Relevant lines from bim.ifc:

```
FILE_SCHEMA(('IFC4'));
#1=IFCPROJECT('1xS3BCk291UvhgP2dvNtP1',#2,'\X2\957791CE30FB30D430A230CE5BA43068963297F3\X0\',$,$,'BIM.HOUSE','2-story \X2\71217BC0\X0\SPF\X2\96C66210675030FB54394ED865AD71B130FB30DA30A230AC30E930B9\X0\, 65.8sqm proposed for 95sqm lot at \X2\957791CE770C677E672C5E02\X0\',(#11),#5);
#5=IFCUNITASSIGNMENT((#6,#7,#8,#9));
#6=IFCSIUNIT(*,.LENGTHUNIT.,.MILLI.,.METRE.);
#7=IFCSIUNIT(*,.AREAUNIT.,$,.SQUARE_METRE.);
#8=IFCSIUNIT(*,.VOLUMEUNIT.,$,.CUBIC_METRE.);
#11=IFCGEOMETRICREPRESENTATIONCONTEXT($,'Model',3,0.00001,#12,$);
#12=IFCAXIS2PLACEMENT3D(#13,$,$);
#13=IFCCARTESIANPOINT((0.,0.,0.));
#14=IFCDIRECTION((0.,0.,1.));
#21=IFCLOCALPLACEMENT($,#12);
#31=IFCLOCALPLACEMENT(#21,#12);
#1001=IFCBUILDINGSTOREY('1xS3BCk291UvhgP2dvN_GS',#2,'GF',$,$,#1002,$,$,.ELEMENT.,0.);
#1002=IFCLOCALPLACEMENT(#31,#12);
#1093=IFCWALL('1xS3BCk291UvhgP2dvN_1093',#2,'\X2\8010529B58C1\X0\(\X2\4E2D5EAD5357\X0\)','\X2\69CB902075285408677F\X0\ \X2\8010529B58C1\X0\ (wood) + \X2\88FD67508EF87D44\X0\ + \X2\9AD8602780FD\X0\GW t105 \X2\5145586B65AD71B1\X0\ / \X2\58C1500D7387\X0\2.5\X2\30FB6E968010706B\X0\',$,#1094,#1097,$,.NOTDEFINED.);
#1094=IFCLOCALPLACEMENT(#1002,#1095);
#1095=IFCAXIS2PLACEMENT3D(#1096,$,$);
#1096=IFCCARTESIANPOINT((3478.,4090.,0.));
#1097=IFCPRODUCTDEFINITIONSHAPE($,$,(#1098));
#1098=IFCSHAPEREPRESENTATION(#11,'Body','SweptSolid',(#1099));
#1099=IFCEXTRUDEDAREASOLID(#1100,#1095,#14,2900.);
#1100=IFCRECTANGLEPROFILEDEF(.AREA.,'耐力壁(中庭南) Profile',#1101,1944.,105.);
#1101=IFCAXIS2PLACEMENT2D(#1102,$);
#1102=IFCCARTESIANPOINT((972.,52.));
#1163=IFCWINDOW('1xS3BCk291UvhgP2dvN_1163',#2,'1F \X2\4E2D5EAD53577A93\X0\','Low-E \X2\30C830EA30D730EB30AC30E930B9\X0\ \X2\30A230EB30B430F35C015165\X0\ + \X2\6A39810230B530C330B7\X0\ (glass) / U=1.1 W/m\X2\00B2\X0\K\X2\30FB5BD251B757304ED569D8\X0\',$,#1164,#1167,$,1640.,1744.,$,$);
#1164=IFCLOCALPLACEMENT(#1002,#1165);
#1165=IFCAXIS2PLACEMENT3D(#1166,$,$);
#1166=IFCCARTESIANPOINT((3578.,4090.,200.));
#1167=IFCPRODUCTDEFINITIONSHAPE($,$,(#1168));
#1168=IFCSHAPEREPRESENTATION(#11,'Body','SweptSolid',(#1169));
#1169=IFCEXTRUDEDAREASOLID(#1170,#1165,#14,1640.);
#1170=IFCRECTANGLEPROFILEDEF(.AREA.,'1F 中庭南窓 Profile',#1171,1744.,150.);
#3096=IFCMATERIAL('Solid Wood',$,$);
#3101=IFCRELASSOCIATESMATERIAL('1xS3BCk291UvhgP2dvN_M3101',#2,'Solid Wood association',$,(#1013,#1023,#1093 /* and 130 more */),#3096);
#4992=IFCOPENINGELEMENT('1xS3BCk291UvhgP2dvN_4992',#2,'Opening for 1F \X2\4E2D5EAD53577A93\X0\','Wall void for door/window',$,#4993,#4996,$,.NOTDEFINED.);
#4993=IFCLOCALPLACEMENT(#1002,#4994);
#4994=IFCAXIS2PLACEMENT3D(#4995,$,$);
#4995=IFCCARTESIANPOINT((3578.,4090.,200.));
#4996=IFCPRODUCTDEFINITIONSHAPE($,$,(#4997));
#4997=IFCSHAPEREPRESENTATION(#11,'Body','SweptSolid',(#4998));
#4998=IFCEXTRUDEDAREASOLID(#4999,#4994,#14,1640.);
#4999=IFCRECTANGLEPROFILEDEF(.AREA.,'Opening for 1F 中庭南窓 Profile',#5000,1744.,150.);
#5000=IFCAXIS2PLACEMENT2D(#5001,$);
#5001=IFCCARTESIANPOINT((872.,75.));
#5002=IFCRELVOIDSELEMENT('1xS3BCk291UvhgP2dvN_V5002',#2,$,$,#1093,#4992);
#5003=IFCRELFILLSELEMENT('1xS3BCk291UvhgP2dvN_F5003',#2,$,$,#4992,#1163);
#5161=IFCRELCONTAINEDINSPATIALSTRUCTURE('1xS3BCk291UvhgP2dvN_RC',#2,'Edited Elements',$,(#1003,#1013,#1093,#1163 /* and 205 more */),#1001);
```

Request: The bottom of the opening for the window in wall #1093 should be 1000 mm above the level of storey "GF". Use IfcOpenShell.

```python
import numpy as np
import ifcopenshell
import ifcopenshell.api.geometry
import ifcopenshell.geom
import ifcopenshell.util.element
import ifcopenshell.util.placement
import ifcopenshell.util.shape
import ifcopenshell.util.unit

model = ifcopenshell.open("bim.ifc")
unit_scale = ifcopenshell.util.unit.calculate_unit_scale(model)

window = model.by_guid("1xS3BCk291UvhgP2dvN_1163")
opening = window.FillsVoids[0].RelatingOpeningElement
storey = ifcopenshell.util.element.get_container(window, ifc_class="IfcBuildingStorey")
level = ifcopenshell.util.placement.get_local_placement(storey.ObjectPlacement)[2, 3]

# The opening's origin need not be at the sill, so measure its lowest point.
shape = ifcopenshell.geom.create_shape(ifcopenshell.geom.settings(), opening)
bottom = ifcopenshell.util.shape.get_shape_bottom_elevation(shape, shape.geometry) / unit_scale
dz = level + 1000.0 - bottom

shift = np.array([0.0, 0.0, dz])
# The window is not placed relative to its opening, so move both.
for product in (opening, window):
    matrix = ifcopenshell.util.placement.get_local_placement(product.ObjectPlacement)
    matrix[:3, 3] += shift
    ifcopenshell.api.geometry.edit_object_placement(model, product=product, matrix=matrix, is_si=False)

print(f"moved by {dz * unit_scale:+.3f} m")

model.write("bim_updated.ifc")
```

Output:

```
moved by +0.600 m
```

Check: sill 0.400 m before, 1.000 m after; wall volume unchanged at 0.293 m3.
